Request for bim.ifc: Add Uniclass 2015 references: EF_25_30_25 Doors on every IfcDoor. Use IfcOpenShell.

First a look at what the model holds.

```python
import ifcopenshell

model = ifcopenshell.open("bim.ifc")
print(model.schema)
print("classifications:", [c.Name for c in model.by_type("IfcClassification")])
for ifc_class in ("IfcDoor", "IfcRoof", "IfcStair", "IfcWall", "IfcWindow"):
    print(ifc_class, len(model.by_type(ifc_class)))
```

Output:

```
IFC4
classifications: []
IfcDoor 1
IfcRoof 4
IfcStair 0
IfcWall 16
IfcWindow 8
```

```python
import ifcopenshell
import ifcopenshell.api.classification

model = ifcopenshell.open("bim.ifc")

system = ifcopenshell.api.classification.add_classification(model, classification="Uniclass 2015")

codes = {
    "IfcDoor": ("EF_25_30_25", "Doors"),
}
for ifc_class, (code, name) in codes.items():
    products = model.by_type(ifc_class)
    ifcopenshell.api.classification.add_reference(
        model, products=products, classification=system, identification=code, name=name
    )
    print(code, len(products))

model.write("bim-out.ifc")
```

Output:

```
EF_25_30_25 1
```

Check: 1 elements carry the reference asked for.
